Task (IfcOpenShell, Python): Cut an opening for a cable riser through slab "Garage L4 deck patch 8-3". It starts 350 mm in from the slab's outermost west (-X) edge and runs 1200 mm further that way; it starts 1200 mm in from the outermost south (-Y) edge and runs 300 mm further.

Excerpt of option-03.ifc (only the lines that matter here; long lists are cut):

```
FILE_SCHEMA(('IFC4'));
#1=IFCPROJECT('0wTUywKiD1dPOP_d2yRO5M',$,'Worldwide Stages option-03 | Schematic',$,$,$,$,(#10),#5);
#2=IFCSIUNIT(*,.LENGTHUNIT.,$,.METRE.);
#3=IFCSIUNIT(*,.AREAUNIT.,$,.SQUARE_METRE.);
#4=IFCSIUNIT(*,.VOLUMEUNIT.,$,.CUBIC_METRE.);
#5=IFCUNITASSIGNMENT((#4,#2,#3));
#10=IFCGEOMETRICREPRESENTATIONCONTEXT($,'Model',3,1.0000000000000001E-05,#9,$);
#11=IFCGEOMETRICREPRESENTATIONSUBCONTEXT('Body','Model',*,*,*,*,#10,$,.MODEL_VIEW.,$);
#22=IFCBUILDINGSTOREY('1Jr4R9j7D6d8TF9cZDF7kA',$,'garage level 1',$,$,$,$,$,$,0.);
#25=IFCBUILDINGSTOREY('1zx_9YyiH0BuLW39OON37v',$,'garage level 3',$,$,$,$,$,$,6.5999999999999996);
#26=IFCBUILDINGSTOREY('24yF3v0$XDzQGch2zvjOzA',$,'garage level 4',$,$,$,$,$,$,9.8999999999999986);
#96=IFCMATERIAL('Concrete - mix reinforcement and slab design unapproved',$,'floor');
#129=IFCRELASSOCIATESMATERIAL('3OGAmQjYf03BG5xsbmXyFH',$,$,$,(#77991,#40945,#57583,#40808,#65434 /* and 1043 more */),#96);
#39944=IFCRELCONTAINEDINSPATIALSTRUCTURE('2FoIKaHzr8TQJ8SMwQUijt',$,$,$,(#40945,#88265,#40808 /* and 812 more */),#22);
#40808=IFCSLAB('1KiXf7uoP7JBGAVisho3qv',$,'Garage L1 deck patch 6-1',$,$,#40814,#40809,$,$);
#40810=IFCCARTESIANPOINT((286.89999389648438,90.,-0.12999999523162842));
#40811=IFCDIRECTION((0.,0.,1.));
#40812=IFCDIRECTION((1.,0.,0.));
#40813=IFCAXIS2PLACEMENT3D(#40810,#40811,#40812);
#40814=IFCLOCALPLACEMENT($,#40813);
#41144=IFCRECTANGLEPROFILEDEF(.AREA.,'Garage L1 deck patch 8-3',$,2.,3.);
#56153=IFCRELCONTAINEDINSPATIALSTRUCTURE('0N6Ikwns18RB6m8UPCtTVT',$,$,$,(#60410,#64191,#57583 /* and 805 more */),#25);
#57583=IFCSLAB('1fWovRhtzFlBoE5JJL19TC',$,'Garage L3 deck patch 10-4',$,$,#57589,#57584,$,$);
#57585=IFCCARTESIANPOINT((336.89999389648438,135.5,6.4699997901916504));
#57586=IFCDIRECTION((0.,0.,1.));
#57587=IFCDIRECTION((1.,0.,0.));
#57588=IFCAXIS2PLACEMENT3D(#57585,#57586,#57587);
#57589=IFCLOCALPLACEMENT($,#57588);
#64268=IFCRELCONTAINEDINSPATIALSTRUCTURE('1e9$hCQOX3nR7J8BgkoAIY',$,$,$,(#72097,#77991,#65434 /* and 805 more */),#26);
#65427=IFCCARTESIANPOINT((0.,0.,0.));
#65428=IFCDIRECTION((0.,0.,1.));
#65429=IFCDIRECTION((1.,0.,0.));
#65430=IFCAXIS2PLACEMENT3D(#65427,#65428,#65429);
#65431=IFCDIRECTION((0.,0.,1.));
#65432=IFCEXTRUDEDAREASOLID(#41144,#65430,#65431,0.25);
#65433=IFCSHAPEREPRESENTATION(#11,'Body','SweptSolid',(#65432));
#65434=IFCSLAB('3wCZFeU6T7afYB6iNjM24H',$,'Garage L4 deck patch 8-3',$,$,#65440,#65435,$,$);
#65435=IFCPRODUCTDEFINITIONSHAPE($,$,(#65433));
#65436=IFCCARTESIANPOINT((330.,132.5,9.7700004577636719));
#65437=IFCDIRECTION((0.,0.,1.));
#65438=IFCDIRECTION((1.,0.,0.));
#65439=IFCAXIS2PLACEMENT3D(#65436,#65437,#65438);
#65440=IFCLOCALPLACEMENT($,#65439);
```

```python
import numpy as np
import ifcopenshell
import ifcopenshell.api.feature
import ifcopenshell.api.geometry
import ifcopenshell.api.root
import ifcopenshell.geom
import ifcopenshell.util.placement
import ifcopenshell.util.representation
import ifcopenshell.util.shape
import ifcopenshell.util.unit

model = ifcopenshell.open("option-03.ifc")
unit_scale = ifcopenshell.util.unit.calculate_unit_scale(model)
settings = ifcopenshell.geom.settings()


def volume(element):
    """Net volume in cubic metres, openings subtracted."""
    shape = ifcopenshell.geom.create_shape(settings, element)
    return ifcopenshell.util.shape.get_volume(shape.geometry)


slab = model.by_id(65434)
before = volume(slab)

# Extent in the slab's own axes, in metres. The edges named are its -X and -Y sides.
slab_shape = ifcopenshell.geom.create_shape(settings, slab)
vertices = ifcopenshell.util.shape.get_vertices(slab_shape.geometry)
x_min, y_min, bottom = vertices.min(axis=0)
top = vertices[:, 2].max()

opening = ifcopenshell.api.root.create_entity(model, ifc_class="IfcOpeningElement", name="Cable riser opening", predefined_type="OPENING")
context = ifcopenshell.util.representation.get_context(model, "Model", "Body", "MODEL_VIEW")
width, depth = 1.2, 0.3
outline = [(0.0, 0.0), (width, 0.0), (width, depth), (0.0, depth), (0.0, 0.0)]
# Overshoot both faces by 50 mm so the cut is clean.
shape = ifcopenshell.api.geometry.add_slab_representation(
    model, context=context, depth=top - bottom + 0.1, polyline=outline
)
ifcopenshell.api.geometry.assign_representation(model, product=opening, representation=shape)

matrix = ifcopenshell.util.placement.get_local_placement(slab.ObjectPlacement)
matrix[:, 3] = matrix @ np.append(np.array([x_min + 0.35, y_min + 1.2, bottom - 0.05]) / unit_scale, 1.0)
ifcopenshell.api.geometry.edit_object_placement(model, product=opening, matrix=matrix, is_si=False)
ifcopenshell.api.feature.add_feature(model, feature=opening, element=slab)

after = volume(slab)

print(f"slab volume {before:.3f} -> {after:.3f} m3")

model.write("option-03-out.ifc")
```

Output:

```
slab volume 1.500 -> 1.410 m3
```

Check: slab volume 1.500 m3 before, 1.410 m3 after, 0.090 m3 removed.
